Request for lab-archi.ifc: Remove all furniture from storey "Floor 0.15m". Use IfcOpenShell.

First a look at what the model holds.

```python
import ifcopenshell
import ifcopenshell.util.element

model = ifcopenshell.open("lab-archi.ifc")
print(model.schema)
storey = next(s for s in model.by_type("IfcBuildingStorey") if s.Name == "Floor 0.15m")
furniture = [e for e in ifcopenshell.util.element.get_decomposition(storey) if e.is_a("IfcFurnishingElement")]
seen = {}
for e in furniture:
    element_type = ifcopenshell.util.element.get_type(e)
    name = element_type.Name if element_type not in (None, e) else None
    seen[name] = seen.get(name, 0) + 1
for name, count in sorted(seen.items(), key=str):
    print(count, "x", name)
```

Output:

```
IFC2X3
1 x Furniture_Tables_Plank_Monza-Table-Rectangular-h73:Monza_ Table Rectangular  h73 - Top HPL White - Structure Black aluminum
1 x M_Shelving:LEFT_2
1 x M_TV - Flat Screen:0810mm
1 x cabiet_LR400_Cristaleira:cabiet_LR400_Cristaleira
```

```python
import ifcopenshell
import ifcopenshell.api.root
import ifcopenshell.util.element

model = ifcopenshell.open("lab-archi.ifc")

storey = next(s for s in model.by_type("IfcBuildingStorey") if s.Name == "Floor 0.15m")
furniture = [e for e in ifcopenshell.util.element.get_decomposition(storey) if e.is_a("IfcFurnishingElement")]

for e in furniture:
    ifcopenshell.api.root.remove_product(model, product=e)
print(len(furniture), "removed")

model.write("lab-archi_edited.ifc")
```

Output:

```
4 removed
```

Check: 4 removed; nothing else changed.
